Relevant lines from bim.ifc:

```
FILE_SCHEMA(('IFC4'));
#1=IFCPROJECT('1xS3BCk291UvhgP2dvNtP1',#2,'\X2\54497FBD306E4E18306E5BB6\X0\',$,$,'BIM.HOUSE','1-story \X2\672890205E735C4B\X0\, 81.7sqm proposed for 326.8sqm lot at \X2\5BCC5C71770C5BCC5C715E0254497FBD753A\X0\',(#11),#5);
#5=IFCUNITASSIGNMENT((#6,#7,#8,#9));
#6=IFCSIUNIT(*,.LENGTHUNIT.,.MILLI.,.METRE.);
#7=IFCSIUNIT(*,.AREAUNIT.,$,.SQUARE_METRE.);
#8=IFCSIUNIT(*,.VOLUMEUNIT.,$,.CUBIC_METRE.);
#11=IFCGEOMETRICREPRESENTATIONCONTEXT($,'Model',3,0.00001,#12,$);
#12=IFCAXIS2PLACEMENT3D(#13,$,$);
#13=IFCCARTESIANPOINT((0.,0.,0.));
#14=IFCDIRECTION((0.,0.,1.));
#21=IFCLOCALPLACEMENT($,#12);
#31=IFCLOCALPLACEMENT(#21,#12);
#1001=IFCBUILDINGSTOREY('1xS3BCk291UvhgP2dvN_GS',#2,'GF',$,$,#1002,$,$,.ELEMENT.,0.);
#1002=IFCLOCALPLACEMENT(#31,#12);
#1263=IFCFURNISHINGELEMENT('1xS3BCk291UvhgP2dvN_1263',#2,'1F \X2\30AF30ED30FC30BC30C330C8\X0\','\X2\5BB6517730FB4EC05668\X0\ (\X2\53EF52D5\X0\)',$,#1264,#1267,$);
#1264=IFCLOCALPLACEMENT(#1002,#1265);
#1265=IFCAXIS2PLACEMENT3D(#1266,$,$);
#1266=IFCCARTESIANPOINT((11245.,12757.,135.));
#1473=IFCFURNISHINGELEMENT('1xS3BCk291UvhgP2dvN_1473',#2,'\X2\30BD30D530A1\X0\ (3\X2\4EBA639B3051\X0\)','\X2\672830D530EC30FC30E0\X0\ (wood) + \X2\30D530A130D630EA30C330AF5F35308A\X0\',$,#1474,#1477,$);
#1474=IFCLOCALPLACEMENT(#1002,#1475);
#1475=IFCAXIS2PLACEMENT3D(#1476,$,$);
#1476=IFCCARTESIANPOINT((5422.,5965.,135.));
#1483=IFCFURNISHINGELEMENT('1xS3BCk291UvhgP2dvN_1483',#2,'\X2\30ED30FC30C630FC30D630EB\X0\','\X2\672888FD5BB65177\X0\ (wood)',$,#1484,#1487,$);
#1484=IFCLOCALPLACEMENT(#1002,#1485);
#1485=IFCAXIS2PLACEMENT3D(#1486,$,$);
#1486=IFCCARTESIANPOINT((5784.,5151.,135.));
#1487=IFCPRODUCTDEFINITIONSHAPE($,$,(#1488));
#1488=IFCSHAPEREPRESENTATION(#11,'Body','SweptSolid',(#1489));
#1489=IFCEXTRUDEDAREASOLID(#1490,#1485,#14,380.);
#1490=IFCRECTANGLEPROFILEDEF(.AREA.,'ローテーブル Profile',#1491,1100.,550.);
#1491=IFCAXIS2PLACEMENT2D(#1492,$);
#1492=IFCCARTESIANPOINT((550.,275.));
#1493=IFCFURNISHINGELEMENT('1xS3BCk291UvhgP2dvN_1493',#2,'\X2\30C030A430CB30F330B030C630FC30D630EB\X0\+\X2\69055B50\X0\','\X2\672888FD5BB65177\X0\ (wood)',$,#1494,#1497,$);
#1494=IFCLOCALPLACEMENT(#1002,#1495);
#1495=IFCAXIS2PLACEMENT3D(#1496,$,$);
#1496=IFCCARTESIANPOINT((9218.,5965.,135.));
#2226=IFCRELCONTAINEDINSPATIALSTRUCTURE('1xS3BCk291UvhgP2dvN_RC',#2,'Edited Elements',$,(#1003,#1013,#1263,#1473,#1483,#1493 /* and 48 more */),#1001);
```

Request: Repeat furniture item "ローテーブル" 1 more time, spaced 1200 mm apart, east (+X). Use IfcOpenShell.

```python
import numpy as np
import ifcopenshell
import ifcopenshell.api.geometry
import ifcopenshell.api.root
import ifcopenshell.util.element
import ifcopenshell.util.placement
import ifcopenshell.util.unit

model = ifcopenshell.open("bim.ifc")
unit_scale = ifcopenshell.util.unit.calculate_unit_scale(model)


def reuse_history(source, copy):
    """copy_class also copies each property set's owner history, people and application; keep the originals."""
    for rel in copy.IsDefinedBy:
        if rel.is_a("IfcRelDefinesByProperties") and (history := rel.RelatingPropertyDefinition.OwnerHistory):
            rel.RelatingPropertyDefinition.OwnerHistory = source.OwnerHistory
            ifcopenshell.util.element.remove_deep2(model, history)


source = model.by_guid("1xS3BCk291UvhgP2dvN_1483")
base = ifcopenshell.util.placement.get_local_placement(source.ObjectPlacement)
step = np.array([1.0, 0.0, 0.0]) * 1.2 / unit_scale

for i in range(1, 2):
    copy = ifcopenshell.api.root.copy_class(model, product=source)
    copy.Representation = ifcopenshell.util.element.copy_deep(
        model, source.Representation, exclude=["IfcGeometricRepresentationContext", "IfcRepresentationMap"]
    )
    reuse_history(source, copy)
    matrix = base.copy()
    matrix[:3, 3] += i * step
    print("added at", matrix[:3, 3].round(3) + 0.0)
    ifcopenshell.api.geometry.edit_object_placement(model, product=copy, matrix=matrix, is_si=False)

model.write("bim_edited.ifc")
```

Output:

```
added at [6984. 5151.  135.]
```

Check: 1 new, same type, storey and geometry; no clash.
